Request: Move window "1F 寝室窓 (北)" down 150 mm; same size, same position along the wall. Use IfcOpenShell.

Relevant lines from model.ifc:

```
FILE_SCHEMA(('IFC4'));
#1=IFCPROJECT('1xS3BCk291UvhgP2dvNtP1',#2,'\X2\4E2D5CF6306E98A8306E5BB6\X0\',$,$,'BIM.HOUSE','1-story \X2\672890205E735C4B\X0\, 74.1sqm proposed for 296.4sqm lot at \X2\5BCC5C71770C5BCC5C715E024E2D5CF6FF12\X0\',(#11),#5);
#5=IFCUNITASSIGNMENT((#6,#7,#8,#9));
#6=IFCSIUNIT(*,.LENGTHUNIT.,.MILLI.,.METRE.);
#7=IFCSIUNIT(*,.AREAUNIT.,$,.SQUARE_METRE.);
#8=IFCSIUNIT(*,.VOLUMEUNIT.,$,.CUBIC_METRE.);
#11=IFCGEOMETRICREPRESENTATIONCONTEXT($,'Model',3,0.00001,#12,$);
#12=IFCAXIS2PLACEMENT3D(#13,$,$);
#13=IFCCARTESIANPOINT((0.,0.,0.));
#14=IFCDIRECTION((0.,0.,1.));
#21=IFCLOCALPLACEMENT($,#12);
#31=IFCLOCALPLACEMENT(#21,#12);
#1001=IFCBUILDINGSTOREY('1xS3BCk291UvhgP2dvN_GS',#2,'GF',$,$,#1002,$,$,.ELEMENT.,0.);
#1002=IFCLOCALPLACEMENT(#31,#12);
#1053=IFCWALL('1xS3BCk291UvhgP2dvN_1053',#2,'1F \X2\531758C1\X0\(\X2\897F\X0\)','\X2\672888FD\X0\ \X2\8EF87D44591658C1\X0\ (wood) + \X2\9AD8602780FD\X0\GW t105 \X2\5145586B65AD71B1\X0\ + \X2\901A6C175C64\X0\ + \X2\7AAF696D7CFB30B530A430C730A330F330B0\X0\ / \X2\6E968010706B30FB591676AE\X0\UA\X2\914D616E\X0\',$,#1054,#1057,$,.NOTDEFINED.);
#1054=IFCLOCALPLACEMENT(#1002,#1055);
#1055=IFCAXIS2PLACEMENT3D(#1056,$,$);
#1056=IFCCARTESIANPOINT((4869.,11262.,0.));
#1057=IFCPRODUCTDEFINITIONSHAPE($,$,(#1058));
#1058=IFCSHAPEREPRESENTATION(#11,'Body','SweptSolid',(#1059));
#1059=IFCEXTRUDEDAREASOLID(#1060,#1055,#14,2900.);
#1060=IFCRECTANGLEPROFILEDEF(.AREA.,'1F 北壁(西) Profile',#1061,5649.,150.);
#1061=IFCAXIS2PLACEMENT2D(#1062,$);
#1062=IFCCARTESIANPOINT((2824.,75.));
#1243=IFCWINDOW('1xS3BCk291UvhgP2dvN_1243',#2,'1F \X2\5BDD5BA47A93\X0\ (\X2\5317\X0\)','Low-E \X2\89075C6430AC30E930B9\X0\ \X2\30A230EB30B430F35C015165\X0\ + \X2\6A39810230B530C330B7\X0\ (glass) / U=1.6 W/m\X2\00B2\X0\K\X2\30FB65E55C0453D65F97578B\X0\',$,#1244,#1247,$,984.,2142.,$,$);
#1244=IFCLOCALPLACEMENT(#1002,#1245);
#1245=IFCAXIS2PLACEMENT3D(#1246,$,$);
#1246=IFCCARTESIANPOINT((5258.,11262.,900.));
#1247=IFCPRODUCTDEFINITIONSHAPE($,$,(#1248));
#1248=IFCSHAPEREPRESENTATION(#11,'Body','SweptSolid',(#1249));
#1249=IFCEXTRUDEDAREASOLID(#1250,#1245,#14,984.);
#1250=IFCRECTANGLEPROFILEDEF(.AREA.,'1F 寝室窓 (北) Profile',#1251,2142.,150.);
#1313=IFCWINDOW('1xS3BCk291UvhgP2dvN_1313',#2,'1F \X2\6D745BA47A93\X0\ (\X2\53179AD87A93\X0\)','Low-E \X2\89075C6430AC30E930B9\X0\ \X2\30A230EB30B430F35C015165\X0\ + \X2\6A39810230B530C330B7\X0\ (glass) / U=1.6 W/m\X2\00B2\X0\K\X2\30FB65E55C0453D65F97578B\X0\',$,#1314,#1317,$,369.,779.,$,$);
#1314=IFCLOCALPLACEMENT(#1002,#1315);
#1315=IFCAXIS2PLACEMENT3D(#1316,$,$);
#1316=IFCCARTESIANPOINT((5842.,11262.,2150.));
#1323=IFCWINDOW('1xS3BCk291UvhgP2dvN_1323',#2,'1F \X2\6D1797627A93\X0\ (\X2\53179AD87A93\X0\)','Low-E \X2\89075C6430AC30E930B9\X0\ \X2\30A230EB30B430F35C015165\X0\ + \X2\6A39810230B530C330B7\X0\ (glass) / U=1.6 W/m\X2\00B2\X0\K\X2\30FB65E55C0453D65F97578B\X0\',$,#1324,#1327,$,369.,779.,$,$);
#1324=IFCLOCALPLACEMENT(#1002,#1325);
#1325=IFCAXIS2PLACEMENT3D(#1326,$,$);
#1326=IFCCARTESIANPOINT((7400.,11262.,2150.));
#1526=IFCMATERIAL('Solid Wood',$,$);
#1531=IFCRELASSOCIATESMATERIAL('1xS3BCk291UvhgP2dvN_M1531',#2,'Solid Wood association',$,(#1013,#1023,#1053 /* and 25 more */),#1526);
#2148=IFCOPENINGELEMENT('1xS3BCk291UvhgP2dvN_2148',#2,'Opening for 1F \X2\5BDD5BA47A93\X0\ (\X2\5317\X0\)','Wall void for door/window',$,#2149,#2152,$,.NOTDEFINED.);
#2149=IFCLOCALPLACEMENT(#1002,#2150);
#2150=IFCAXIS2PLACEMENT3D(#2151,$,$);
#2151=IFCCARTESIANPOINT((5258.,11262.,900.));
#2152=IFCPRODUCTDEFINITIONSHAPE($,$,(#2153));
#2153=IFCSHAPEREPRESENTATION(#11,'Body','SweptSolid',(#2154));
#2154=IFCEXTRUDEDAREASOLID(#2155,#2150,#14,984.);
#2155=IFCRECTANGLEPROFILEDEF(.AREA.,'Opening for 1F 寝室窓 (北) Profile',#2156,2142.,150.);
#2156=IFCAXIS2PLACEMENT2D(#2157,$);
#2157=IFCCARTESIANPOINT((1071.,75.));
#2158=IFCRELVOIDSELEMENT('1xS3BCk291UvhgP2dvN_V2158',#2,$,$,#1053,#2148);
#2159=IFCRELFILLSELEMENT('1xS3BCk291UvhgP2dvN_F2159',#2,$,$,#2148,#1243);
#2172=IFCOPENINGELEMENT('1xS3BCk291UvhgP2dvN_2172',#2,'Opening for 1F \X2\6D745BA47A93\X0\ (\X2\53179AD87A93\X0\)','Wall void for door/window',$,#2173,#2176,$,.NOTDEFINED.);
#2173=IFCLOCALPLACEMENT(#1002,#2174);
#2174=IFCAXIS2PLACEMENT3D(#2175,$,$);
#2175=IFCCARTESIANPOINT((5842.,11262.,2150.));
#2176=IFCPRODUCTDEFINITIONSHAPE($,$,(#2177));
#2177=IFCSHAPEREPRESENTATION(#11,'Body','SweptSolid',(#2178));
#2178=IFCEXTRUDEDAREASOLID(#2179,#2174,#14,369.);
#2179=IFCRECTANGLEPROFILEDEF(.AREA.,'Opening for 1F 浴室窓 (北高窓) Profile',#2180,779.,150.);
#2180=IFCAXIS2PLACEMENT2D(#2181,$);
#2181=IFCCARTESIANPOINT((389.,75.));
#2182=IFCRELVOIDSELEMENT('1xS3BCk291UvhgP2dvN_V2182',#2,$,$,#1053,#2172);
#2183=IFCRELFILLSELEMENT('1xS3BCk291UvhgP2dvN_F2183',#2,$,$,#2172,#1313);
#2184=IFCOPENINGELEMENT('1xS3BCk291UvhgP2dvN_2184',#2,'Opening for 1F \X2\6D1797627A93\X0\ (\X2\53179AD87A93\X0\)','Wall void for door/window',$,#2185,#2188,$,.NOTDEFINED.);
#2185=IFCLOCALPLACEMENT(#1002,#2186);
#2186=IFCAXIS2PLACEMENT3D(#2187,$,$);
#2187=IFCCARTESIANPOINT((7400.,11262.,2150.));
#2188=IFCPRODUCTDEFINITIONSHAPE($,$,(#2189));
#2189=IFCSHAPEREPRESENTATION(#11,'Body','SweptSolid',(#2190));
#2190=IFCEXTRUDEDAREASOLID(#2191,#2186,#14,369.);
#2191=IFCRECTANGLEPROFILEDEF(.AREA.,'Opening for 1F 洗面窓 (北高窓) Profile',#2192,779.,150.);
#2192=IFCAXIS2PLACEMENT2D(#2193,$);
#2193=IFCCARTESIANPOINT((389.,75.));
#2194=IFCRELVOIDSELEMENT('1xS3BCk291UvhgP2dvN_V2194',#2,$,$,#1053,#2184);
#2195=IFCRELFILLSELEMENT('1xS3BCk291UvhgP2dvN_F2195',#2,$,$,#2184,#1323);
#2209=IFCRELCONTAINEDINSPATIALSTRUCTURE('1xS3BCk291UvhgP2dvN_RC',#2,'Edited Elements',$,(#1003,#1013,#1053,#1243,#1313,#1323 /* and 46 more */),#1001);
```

```python
import numpy as np
import ifcopenshell
import ifcopenshell.api.geometry
import ifcopenshell.util.placement
import ifcopenshell.util.unit

model = ifcopenshell.open("model.ifc")
unit_scale = ifcopenshell.util.unit.calculate_unit_scale(model)

window = model.by_id(1243)
opening = window.FillsVoids[0].RelatingOpeningElement
dz = -150.0

shift = np.array([0.0, 0.0, dz])
# The window is not placed relative to its opening, so move both.
for product in (opening, window):
    matrix = ifcopenshell.util.placement.get_local_placement(product.ObjectPlacement)
    matrix[:3, 3] += shift
    ifcopenshell.api.geometry.edit_object_placement(model, product=product, matrix=matrix, is_si=False)

print(f"moved by {dz * unit_scale:+.3f} m")

model.write("model_edited.ifc")
```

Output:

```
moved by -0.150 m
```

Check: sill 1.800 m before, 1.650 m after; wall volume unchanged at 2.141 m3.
